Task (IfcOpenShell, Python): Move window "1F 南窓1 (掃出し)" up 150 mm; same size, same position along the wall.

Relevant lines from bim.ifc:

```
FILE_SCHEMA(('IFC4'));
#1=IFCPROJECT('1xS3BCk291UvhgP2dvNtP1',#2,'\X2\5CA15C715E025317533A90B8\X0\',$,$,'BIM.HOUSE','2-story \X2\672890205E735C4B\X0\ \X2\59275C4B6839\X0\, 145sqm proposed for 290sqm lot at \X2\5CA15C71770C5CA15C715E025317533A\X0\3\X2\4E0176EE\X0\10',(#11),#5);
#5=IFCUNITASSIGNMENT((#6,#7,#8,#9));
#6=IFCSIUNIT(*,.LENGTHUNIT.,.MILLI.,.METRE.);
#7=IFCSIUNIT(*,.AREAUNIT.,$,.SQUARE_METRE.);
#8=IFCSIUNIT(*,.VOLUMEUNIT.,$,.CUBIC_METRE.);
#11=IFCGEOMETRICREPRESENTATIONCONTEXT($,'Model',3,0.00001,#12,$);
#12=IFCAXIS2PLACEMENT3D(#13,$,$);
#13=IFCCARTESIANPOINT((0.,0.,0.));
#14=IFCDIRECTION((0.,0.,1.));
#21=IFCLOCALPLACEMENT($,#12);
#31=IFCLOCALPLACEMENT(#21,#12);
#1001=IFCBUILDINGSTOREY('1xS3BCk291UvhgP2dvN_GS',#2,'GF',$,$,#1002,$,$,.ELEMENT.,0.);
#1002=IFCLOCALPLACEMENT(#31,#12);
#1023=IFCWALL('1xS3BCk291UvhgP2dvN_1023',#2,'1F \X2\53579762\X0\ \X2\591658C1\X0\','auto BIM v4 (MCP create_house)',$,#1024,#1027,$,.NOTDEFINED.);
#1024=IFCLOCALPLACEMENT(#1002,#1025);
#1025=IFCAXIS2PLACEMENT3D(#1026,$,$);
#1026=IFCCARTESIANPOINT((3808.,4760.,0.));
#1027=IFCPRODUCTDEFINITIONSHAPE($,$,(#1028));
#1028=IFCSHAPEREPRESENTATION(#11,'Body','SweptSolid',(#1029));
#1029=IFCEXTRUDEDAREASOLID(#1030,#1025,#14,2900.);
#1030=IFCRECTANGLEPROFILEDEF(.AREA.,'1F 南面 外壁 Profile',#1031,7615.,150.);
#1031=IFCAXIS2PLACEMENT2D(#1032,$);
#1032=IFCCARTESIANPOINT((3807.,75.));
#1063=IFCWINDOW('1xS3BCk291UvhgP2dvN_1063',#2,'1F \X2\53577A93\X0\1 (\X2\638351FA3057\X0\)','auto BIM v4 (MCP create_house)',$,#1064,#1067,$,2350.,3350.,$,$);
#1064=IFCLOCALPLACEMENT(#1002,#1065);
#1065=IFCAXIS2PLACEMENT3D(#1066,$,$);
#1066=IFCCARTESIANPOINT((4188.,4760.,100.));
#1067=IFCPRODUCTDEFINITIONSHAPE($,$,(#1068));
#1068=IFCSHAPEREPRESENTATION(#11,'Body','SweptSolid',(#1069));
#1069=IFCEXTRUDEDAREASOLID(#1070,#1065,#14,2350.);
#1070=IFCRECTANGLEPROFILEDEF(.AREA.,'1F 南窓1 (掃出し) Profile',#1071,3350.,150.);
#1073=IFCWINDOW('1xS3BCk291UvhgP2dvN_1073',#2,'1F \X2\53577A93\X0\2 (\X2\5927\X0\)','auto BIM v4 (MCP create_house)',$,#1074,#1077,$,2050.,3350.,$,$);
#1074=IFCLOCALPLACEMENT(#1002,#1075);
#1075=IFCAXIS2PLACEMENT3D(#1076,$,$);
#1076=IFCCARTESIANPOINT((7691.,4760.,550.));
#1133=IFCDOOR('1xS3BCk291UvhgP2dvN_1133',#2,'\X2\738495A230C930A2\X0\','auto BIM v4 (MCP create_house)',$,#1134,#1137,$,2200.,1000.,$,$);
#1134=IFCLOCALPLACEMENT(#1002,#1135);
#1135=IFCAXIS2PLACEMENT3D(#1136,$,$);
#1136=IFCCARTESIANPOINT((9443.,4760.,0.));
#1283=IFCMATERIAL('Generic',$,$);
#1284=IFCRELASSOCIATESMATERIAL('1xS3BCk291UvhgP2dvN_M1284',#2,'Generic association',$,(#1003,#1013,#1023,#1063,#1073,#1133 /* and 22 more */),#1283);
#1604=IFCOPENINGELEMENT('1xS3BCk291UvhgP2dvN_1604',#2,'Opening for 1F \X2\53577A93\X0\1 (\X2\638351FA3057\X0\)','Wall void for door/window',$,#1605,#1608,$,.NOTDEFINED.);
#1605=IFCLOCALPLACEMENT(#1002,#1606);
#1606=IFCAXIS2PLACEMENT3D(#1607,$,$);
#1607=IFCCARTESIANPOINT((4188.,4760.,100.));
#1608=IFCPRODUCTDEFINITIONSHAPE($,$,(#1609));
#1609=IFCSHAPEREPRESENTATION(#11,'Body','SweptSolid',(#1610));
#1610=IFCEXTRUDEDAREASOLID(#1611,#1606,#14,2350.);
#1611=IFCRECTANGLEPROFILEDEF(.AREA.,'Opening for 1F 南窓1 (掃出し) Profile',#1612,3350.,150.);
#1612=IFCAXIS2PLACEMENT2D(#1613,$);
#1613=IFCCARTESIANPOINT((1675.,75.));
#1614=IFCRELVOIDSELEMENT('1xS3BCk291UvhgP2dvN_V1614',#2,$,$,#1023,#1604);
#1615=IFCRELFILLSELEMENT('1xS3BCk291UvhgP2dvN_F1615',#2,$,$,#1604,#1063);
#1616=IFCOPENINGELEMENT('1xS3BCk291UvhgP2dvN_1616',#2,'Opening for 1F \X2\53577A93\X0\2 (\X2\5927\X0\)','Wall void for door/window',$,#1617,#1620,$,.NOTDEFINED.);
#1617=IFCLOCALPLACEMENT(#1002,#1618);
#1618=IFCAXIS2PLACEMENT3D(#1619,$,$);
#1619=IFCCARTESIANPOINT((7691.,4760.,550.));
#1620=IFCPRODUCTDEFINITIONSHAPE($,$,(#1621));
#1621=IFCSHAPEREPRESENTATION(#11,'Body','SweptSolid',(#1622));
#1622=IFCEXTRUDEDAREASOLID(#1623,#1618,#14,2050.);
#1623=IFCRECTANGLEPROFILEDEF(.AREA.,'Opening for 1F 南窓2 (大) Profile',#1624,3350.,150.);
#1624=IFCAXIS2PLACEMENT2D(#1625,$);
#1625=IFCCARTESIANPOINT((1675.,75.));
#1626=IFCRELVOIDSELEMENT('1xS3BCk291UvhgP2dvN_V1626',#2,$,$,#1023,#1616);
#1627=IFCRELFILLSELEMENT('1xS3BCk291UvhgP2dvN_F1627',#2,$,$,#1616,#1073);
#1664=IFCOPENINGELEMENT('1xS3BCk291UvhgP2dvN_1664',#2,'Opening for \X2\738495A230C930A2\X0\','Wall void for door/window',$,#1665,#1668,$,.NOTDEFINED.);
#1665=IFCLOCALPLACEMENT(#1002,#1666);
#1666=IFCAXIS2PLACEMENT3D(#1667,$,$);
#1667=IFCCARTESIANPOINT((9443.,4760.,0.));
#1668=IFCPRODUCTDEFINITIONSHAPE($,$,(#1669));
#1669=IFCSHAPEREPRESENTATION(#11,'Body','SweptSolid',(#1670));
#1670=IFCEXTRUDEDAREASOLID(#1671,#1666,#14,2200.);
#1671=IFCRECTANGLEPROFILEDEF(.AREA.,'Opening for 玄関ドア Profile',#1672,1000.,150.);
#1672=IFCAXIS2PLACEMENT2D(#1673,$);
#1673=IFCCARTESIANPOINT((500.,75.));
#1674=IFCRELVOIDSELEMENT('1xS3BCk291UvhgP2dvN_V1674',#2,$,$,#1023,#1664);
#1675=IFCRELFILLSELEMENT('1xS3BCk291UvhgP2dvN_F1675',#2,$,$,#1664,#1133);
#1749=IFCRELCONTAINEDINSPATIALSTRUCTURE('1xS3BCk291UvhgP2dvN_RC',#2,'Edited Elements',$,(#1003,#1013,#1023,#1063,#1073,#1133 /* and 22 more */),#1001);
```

```python
import numpy as np
import ifcopenshell
import ifcopenshell.api.geometry
import ifcopenshell.util.placement
import ifcopenshell.util.unit

model = ifcopenshell.open("bim.ifc")
unit_scale = ifcopenshell.util.unit.calculate_unit_scale(model)

window = model.by_id(1063)
opening = window.FillsVoids[0].RelatingOpeningElement
dz = 0.15 / unit_scale

shift = np.array([0.0, 0.0, dz])
# The window is not placed relative to its opening, so move both.
for product in (opening, window):
    matrix = ifcopenshell.util.placement.get_local_placement(product.ObjectPlacement)
    matrix[:3, 3] += shift
    ifcopenshell.api.geometry.edit_object_placement(model, product=product, matrix=matrix, is_si=False)

print(f"moved by {dz * unit_scale:+.3f} m")

model.write("bim_v2.ifc")
```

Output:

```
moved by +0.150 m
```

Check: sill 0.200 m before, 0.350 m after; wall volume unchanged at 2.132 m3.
